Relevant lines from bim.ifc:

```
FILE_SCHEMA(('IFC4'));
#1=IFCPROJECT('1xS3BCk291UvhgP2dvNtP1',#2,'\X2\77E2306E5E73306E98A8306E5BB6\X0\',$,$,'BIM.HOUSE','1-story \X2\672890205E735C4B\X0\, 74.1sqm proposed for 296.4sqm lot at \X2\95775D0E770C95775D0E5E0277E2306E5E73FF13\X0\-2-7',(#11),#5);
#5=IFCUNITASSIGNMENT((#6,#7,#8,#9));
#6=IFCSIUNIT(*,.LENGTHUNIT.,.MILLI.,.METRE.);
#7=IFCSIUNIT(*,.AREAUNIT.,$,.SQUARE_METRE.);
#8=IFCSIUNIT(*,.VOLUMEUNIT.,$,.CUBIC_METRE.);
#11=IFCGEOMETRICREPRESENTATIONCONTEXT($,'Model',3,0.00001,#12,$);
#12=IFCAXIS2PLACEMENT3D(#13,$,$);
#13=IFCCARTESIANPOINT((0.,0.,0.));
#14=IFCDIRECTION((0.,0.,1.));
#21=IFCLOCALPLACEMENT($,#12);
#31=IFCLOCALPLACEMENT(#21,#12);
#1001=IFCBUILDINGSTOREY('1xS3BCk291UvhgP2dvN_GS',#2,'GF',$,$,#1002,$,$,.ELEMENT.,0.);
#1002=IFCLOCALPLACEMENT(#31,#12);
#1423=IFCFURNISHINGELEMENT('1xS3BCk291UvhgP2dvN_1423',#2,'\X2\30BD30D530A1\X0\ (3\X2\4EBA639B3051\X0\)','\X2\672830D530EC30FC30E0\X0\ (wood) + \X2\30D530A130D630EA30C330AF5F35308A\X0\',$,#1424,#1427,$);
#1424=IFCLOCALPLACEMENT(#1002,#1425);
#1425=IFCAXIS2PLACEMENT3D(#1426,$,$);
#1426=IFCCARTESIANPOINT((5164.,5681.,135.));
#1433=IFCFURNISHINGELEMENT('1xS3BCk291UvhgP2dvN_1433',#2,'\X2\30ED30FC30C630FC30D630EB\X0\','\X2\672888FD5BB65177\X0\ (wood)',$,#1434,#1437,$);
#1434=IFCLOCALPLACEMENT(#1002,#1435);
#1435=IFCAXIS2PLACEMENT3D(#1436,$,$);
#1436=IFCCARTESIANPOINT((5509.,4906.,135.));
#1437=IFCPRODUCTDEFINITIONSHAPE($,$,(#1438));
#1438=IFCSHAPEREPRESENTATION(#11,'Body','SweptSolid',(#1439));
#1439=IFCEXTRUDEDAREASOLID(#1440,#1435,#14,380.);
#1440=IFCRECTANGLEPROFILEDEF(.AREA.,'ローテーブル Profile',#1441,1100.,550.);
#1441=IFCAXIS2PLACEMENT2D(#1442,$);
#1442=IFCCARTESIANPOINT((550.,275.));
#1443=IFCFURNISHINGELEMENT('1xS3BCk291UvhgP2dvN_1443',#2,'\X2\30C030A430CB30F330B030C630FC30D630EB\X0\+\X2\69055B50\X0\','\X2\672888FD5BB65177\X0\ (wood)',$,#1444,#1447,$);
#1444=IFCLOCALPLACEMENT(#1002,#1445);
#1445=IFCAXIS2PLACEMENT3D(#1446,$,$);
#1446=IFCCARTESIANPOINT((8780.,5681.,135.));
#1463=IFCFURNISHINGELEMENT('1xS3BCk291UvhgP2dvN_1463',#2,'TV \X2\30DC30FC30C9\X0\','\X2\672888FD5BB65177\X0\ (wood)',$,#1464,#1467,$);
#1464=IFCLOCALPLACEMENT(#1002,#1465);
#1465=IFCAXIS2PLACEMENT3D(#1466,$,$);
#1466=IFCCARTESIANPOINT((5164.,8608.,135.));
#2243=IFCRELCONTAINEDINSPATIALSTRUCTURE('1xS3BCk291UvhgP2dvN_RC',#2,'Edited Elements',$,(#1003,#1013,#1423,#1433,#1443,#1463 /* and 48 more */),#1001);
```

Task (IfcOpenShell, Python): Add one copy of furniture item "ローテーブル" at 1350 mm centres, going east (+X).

```python
import numpy as np
import ifcopenshell
import ifcopenshell.api.geometry
import ifcopenshell.api.root
import ifcopenshell.util.element
import ifcopenshell.util.placement
import ifcopenshell.util.unit

model = ifcopenshell.open("bim.ifc")
unit_scale = ifcopenshell.util.unit.calculate_unit_scale(model)


def reuse_history(source, copy):
    """copy_class also copies each property set's owner history, people and application; keep the originals."""
    for rel in copy.IsDefinedBy:
        if rel.is_a("IfcRelDefinesByProperties") and (history := rel.RelatingPropertyDefinition.OwnerHistory):
            rel.RelatingPropertyDefinition.OwnerHistory = source.OwnerHistory
            ifcopenshell.util.element.remove_deep2(model, history)


source = model.by_guid("1xS3BCk291UvhgP2dvN_1433")
base = ifcopenshell.util.placement.get_local_placement(source.ObjectPlacement)
step = np.array([1.0, 0.0, 0.0]) * 1.35 / unit_scale

for i in range(1, 2):
    copy = ifcopenshell.api.root.copy_class(model, product=source)
    copy.Representation = ifcopenshell.util.element.copy_deep(
        model, source.Representation, exclude=["IfcGeometricRepresentationContext", "IfcRepresentationMap"]
    )
    reuse_history(source, copy)
    matrix = base.copy()
    matrix[:3, 3] += i * step
    print("added at", matrix[:3, 3].round(3) + 0.0)
    ifcopenshell.api.geometry.edit_object_placement(model, product=copy, matrix=matrix, is_si=False)

model.write("bim_v2.ifc")
```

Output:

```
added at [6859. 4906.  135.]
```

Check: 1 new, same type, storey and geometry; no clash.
